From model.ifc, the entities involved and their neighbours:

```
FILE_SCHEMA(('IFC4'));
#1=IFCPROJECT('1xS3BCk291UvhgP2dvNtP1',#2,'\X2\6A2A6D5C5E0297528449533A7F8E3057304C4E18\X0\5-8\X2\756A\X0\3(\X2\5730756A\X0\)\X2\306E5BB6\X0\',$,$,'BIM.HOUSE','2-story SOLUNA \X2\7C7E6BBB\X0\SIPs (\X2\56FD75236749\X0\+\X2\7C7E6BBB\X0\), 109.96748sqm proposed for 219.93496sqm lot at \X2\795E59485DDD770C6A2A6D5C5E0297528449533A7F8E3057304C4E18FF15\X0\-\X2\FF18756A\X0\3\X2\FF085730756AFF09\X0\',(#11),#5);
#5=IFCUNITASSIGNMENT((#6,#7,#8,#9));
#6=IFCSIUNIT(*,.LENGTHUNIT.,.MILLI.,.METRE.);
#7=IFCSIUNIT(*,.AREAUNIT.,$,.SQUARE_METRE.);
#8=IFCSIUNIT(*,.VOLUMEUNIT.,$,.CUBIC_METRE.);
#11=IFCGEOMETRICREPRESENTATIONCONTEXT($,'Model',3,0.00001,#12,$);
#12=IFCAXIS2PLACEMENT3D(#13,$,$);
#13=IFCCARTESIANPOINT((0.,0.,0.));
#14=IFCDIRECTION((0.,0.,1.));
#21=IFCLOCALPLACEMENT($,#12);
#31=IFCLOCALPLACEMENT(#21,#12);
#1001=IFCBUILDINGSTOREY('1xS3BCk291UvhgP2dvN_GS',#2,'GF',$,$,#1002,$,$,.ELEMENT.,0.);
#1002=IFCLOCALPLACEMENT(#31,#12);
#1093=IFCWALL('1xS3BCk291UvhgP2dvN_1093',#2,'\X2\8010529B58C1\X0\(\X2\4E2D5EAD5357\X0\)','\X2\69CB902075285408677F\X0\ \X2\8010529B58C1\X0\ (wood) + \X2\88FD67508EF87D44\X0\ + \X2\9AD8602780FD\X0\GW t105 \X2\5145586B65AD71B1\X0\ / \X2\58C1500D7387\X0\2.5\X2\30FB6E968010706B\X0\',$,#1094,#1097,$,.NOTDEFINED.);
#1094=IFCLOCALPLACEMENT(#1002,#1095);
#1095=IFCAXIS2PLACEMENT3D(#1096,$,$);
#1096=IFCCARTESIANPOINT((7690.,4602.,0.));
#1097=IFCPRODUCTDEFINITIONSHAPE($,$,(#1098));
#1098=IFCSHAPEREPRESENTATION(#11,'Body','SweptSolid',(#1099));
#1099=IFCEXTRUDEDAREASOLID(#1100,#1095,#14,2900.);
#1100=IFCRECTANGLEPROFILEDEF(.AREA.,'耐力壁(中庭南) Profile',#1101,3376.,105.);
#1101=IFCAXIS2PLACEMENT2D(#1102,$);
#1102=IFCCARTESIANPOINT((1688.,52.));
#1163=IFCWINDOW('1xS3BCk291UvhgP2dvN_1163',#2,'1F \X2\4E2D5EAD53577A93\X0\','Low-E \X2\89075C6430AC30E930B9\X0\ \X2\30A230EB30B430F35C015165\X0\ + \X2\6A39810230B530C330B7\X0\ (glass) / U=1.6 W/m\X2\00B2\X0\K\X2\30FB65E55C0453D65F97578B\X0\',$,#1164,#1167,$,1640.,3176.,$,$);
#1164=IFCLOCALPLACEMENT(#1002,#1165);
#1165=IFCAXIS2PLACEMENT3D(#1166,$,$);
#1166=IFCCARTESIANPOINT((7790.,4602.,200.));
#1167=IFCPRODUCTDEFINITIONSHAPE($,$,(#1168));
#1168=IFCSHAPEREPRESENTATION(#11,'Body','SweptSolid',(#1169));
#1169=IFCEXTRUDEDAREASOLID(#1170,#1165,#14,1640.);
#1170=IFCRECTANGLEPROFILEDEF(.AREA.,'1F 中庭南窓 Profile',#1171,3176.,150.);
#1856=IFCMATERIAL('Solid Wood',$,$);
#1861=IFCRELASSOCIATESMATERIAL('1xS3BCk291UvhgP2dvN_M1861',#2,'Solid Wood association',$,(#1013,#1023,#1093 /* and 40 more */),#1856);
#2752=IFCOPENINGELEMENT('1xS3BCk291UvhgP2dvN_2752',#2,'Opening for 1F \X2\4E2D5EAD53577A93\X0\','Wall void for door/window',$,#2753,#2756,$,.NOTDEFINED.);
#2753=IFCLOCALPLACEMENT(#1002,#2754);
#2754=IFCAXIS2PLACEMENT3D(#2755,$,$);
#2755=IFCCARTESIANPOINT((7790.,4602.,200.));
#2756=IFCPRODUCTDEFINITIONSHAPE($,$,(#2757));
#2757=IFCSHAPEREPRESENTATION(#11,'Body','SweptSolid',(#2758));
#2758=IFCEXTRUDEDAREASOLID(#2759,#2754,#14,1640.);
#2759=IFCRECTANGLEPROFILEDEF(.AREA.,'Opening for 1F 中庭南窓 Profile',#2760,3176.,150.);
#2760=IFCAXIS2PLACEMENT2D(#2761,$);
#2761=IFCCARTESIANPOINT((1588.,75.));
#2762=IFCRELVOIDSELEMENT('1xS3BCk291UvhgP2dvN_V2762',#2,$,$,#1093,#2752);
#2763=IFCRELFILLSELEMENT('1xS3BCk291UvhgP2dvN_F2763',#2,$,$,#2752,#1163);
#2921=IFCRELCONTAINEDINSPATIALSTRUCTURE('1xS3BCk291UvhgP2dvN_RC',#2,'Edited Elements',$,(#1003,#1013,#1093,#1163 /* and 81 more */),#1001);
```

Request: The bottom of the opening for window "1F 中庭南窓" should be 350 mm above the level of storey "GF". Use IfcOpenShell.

```python
import numpy as np
import ifcopenshell
import ifcopenshell.api.geometry
import ifcopenshell.geom
import ifcopenshell.util.element
import ifcopenshell.util.placement
import ifcopenshell.util.shape
import ifcopenshell.util.unit

model = ifcopenshell.open("model.ifc")
unit_scale = ifcopenshell.util.unit.calculate_unit_scale(model)

window = model.by_guid("1xS3BCk291UvhgP2dvN_1163")
opening = window.FillsVoids[0].RelatingOpeningElement
storey = ifcopenshell.util.element.get_container(window, ifc_class="IfcBuildingStorey")
level = ifcopenshell.util.placement.get_local_placement(storey.ObjectPlacement)[2, 3]

# The opening's origin need not be at the sill, so measure its lowest point.
shape = ifcopenshell.geom.create_shape(ifcopenshell.geom.settings(), opening)
bottom = ifcopenshell.util.shape.get_shape_bottom_elevation(shape, shape.geometry) / unit_scale
dz = level + 0.35 / unit_scale - bottom

shift = np.array([0.0, 0.0, dz])
# The window is not placed relative to its opening, so move both.
for product in (opening, window):
    matrix = ifcopenshell.util.placement.get_local_placement(product.ObjectPlacement)
    matrix[:3, 3] += shift
    ifcopenshell.api.geometry.edit_object_placement(model, product=product, matrix=matrix, is_si=False)

print(f"moved by {dz * unit_scale:+.3f} m")

model.write("model-out.ifc")
```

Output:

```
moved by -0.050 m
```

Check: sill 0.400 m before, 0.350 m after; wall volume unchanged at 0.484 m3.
